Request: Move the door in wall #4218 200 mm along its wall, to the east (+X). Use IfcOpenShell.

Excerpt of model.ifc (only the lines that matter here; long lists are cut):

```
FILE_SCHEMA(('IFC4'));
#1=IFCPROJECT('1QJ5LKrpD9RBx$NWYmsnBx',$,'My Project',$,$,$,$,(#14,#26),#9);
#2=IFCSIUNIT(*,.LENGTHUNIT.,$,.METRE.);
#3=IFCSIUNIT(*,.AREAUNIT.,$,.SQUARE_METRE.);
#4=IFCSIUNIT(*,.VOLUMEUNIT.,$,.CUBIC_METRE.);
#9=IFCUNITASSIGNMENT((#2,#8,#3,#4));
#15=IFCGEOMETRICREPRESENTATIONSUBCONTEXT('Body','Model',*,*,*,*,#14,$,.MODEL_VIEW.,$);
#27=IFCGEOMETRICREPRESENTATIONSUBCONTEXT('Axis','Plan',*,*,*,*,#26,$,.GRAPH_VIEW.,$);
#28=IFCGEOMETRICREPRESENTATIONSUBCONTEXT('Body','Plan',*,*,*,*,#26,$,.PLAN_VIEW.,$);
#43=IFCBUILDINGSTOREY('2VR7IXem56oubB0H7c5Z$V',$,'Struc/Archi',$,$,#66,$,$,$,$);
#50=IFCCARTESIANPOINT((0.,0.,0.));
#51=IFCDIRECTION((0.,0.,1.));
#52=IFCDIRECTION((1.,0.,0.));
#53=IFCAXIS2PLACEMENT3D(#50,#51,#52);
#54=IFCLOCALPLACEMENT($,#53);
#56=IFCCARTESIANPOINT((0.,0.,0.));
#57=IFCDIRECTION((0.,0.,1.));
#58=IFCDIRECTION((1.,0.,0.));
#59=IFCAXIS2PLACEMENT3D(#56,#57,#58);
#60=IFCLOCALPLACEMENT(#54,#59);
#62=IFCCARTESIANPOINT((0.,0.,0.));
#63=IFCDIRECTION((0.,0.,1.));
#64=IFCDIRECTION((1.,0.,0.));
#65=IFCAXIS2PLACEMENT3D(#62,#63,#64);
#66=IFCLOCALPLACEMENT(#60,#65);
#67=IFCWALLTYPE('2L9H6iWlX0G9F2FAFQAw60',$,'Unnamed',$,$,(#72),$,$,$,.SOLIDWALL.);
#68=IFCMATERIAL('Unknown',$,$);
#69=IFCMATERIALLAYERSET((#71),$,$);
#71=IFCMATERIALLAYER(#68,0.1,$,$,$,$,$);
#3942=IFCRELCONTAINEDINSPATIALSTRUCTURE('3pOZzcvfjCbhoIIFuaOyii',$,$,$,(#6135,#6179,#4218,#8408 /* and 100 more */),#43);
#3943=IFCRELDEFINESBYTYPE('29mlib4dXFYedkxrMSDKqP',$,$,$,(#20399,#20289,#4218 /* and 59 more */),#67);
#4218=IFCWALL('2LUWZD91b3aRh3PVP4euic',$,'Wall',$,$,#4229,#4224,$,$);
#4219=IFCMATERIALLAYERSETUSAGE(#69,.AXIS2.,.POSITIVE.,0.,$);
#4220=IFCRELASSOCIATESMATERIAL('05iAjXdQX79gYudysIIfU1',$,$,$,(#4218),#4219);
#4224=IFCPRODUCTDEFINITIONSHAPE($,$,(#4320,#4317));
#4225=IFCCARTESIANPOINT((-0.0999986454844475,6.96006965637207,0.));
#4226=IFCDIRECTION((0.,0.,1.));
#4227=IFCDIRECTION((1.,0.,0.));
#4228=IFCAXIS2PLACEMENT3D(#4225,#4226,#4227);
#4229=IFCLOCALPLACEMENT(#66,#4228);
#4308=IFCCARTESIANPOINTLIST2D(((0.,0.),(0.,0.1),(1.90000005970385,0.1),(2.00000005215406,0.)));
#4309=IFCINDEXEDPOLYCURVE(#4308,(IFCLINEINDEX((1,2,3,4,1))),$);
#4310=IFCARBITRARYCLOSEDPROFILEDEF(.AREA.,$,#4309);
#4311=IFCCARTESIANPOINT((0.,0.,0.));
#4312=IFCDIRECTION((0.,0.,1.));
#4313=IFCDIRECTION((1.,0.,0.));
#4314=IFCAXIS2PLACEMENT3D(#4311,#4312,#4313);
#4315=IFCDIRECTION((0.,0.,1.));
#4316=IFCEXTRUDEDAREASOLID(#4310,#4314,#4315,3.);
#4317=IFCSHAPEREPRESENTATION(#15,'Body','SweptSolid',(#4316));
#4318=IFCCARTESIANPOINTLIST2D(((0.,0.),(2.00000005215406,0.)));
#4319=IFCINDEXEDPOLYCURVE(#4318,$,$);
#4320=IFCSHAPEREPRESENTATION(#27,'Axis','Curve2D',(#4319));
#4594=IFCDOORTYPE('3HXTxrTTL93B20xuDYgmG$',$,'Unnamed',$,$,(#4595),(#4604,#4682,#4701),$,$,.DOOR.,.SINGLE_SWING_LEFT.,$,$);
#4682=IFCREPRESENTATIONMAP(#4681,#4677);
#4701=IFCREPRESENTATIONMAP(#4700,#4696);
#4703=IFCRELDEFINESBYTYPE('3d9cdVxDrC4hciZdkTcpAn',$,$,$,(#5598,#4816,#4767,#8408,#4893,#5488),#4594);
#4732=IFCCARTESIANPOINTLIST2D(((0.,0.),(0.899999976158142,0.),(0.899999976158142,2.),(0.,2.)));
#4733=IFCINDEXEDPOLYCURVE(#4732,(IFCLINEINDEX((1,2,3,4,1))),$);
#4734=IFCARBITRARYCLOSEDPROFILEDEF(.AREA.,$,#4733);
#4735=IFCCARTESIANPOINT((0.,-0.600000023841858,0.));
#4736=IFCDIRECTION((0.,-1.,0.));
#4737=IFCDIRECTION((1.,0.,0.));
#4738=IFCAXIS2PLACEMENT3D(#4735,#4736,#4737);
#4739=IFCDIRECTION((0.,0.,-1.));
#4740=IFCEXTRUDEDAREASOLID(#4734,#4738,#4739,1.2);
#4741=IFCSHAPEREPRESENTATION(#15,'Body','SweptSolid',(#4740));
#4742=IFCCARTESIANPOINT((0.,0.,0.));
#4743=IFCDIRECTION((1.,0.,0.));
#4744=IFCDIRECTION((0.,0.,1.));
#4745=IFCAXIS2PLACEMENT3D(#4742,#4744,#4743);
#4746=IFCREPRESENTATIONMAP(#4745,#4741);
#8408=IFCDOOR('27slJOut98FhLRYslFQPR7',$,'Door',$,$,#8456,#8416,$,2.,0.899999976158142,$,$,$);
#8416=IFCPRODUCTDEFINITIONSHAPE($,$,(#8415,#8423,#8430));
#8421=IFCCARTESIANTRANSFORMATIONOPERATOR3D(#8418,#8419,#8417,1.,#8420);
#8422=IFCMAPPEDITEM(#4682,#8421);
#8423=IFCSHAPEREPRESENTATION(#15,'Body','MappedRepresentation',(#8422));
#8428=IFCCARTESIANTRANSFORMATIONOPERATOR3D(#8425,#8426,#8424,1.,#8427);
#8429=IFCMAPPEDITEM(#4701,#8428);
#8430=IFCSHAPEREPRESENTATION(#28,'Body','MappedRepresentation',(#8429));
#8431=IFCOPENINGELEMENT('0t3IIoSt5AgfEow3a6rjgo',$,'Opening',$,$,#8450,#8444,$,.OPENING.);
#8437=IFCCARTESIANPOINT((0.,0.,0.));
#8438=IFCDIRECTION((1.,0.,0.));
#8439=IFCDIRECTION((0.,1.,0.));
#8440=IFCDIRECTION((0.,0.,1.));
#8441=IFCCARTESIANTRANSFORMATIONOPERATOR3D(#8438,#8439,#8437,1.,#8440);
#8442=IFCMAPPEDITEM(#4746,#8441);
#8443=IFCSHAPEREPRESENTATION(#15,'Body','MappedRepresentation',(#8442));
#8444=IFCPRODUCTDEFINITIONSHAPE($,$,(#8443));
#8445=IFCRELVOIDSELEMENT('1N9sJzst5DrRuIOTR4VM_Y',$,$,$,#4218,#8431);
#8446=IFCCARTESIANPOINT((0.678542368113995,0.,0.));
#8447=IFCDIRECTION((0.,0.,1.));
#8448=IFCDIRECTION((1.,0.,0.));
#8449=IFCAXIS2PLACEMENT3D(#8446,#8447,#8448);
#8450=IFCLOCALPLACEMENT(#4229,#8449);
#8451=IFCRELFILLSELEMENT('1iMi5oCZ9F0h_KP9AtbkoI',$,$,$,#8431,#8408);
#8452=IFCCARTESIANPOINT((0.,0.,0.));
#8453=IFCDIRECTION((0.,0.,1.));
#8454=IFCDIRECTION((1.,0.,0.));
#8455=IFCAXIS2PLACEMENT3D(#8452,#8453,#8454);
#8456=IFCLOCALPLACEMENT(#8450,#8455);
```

```python
import ifcopenshell
import ifcopenshell.api.geometry
import ifcopenshell.util.placement
import ifcopenshell.util.unit

model = ifcopenshell.open("model.ifc")
unit_scale = ifcopenshell.util.unit.calculate_unit_scale(model)

door = model.by_guid("27slJOut98FhLRYslFQPR7")
opening = door.FillsVoids[0].RelatingOpeningElement
wall = opening.VoidsElements[0].RelatingBuildingElement

wall_matrix = ifcopenshell.util.placement.get_local_placement(wall.ObjectPlacement)
shift = wall_matrix[:3, 0] * 0.2 / unit_scale
before = ifcopenshell.util.placement.get_local_placement(door.ObjectPlacement)[:3, 3].copy()

# The door is placed relative to its opening, so it follows when the opening moves.
matrix = ifcopenshell.util.placement.get_local_placement(opening.ObjectPlacement)
matrix[:3, 3] += shift
ifcopenshell.api.geometry.edit_object_placement(
    model, product=opening, matrix=matrix, is_si=False, should_transform_children=True
)

after = ifcopenshell.util.placement.get_local_placement(door.ObjectPlacement)[:3, 3]
print("door moved by", (after - before).round(3) + 0.0)

model.write("model-out.ifc")
```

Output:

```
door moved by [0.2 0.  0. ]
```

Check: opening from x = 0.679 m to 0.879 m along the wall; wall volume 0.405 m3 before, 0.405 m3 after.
